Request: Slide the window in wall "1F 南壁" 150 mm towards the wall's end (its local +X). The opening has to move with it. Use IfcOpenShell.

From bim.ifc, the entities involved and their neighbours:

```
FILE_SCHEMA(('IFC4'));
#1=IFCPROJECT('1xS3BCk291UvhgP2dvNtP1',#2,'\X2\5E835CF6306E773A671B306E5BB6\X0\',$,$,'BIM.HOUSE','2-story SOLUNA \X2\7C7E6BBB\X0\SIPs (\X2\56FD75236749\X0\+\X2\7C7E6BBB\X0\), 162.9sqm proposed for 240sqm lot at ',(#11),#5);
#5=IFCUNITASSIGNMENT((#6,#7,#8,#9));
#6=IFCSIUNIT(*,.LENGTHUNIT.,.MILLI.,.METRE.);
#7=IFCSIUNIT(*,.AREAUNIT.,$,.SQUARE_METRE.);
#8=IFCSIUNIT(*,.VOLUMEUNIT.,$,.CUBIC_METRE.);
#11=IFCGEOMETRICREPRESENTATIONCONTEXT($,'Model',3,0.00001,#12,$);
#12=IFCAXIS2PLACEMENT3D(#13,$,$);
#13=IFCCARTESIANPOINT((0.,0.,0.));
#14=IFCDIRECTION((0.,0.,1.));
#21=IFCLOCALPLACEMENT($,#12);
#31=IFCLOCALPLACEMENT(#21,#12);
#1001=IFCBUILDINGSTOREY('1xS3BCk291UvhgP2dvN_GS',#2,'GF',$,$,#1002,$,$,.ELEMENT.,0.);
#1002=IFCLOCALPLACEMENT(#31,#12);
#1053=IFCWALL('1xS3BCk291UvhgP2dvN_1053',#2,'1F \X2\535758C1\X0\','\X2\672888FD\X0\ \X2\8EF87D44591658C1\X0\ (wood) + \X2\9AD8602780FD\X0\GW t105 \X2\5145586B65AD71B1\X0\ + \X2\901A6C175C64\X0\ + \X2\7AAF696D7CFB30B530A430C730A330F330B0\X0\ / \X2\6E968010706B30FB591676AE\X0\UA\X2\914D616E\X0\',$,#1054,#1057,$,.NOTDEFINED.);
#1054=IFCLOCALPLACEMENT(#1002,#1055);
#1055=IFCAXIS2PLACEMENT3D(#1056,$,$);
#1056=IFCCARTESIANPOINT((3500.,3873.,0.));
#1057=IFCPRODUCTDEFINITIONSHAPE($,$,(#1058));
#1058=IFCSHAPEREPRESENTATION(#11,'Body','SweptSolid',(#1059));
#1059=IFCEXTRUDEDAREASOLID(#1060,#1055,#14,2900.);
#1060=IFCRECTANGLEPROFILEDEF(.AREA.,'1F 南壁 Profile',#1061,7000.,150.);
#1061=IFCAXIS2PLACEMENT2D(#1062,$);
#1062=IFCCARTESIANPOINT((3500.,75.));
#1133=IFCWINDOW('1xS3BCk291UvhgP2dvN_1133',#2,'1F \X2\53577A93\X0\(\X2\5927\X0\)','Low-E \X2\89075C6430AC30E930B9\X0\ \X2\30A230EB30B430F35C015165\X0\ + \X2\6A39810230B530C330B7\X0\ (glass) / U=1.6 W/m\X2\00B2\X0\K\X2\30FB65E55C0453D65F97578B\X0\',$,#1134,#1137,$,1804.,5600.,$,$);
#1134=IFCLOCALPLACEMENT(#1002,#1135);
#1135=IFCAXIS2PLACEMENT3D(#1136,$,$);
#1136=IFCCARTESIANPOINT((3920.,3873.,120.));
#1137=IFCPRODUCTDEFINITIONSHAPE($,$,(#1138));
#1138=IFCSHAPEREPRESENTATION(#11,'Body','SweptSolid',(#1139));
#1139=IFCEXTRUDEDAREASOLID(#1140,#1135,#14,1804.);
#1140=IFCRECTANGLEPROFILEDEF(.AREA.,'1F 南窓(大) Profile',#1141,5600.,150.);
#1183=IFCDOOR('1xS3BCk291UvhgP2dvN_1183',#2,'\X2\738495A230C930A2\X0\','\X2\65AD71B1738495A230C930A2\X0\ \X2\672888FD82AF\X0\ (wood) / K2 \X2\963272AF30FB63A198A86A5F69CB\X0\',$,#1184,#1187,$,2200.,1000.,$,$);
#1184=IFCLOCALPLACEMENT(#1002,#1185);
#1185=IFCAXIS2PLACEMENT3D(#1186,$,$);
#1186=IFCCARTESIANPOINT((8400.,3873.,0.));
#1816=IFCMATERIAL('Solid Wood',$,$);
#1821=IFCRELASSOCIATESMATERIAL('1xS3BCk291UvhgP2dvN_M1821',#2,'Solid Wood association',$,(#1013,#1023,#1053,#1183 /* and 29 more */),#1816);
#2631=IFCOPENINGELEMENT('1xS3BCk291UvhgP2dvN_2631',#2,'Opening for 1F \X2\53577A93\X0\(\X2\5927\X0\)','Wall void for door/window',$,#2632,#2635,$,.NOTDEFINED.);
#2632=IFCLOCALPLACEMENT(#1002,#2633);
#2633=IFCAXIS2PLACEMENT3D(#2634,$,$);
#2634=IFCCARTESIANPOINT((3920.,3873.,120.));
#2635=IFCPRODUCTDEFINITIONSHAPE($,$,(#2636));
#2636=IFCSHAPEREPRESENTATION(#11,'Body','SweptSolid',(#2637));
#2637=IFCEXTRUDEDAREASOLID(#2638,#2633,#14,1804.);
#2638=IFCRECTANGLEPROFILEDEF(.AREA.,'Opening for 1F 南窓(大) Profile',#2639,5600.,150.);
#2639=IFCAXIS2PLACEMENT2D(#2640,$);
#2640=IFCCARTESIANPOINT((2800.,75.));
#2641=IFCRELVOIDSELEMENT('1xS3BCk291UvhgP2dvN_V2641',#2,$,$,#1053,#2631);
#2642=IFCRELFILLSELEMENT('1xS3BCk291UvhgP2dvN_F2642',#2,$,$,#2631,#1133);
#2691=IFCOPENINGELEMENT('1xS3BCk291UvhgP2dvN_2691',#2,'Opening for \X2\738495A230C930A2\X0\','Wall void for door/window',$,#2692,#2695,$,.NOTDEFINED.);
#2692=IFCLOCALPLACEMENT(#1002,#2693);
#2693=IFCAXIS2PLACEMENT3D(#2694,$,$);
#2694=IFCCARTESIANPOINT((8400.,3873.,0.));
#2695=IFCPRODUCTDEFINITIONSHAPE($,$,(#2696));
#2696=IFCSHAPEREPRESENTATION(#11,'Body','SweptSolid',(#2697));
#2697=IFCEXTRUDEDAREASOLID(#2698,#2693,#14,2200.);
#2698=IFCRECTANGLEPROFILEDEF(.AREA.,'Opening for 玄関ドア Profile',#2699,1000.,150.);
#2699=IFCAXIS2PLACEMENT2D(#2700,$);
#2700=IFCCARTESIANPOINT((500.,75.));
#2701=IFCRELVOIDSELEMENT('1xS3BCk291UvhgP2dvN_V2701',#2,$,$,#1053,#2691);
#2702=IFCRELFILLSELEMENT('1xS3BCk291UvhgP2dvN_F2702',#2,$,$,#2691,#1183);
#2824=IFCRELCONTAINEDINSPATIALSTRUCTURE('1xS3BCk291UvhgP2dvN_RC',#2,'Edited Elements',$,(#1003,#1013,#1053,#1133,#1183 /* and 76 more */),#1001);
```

```python
import ifcopenshell
import ifcopenshell.api.geometry
import ifcopenshell.util.placement
import ifcopenshell.util.unit

model = ifcopenshell.open("bim.ifc")
unit_scale = ifcopenshell.util.unit.calculate_unit_scale(model)

window = model.by_id(1133)
opening = window.FillsVoids[0].RelatingOpeningElement
wall = opening.VoidsElements[0].RelatingBuildingElement

wall_matrix = ifcopenshell.util.placement.get_local_placement(wall.ObjectPlacement)
shift = wall_matrix[:3, 0] * 0.15 / unit_scale
before = ifcopenshell.util.placement.get_local_placement(window.ObjectPlacement)[:3, 3].copy()

# The window is not placed relative to its opening, so move both.
for product in (opening, window):
    matrix = ifcopenshell.util.placement.get_local_placement(product.ObjectPlacement)
    matrix[:3, 3] += shift
    ifcopenshell.api.geometry.edit_object_placement(model, product=product, matrix=matrix, is_si=False)

after = ifcopenshell.util.placement.get_local_placement(window.ObjectPlacement)[:3, 3]
print("window moved by", (after - before).round(3) + 0.0)

model.write("bim_edited.ifc")
```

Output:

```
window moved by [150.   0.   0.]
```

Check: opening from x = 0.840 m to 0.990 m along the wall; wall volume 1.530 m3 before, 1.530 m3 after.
